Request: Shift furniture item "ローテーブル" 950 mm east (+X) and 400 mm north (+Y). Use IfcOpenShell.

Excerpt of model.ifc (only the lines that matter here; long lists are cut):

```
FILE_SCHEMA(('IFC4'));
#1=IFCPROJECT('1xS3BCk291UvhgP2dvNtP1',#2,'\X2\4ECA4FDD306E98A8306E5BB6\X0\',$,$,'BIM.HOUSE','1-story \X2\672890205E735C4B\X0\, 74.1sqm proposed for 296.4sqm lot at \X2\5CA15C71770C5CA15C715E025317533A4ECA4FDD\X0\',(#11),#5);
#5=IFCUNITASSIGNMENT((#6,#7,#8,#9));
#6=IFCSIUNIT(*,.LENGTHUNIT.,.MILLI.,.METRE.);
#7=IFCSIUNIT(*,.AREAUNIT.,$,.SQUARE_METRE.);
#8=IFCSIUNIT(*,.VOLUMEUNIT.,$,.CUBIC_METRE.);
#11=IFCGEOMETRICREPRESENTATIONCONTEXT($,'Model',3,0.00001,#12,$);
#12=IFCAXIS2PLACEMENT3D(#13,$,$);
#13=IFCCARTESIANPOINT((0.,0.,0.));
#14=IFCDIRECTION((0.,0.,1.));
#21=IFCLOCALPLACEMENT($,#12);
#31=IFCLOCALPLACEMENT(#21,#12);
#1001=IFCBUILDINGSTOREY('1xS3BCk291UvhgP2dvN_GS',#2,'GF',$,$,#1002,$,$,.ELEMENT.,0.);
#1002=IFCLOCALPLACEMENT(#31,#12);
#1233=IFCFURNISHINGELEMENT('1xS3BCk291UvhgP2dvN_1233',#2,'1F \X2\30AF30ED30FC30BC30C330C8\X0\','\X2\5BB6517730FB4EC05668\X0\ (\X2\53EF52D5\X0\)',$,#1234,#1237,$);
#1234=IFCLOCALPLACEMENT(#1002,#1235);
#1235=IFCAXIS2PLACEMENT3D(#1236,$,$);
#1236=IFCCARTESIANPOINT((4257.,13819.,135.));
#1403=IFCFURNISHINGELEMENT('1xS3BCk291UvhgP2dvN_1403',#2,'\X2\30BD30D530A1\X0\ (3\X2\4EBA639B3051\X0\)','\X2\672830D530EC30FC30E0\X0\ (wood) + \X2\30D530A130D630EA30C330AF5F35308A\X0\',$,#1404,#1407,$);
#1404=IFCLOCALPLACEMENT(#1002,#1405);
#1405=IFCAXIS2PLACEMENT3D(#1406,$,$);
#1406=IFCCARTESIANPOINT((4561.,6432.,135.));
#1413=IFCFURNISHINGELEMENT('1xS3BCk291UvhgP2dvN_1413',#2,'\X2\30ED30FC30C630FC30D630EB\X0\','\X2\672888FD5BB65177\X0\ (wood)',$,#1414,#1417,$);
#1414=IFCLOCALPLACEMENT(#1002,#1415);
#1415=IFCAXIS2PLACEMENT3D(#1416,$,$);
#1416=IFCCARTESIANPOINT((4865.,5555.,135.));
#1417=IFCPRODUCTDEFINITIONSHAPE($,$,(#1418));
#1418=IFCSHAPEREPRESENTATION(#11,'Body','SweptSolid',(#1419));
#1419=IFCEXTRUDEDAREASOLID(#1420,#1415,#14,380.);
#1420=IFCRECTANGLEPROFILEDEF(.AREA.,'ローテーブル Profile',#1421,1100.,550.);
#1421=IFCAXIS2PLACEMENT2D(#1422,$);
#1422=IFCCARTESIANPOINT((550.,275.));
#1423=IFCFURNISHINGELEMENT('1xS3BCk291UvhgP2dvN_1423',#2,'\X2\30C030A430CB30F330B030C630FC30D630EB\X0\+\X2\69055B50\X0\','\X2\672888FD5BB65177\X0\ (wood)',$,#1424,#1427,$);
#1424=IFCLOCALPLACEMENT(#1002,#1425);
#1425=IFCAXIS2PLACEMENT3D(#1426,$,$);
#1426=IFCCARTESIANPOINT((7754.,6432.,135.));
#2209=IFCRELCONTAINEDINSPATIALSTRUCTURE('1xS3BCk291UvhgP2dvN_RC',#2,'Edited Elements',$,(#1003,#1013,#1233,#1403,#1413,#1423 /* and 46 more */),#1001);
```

```python
import ifcopenshell
import ifcopenshell.api.geometry
import ifcopenshell.util.placement

model = ifcopenshell.open("model.ifc")

item = model.by_id(1413)
matrix = ifcopenshell.util.placement.get_local_placement(item.ObjectPlacement)
matrix[0, 3] += 950.0
matrix[1, 3] += 400.0
ifcopenshell.api.geometry.edit_object_placement(model, product=item, matrix=matrix, is_si=False)

print(ifcopenshell.util.placement.get_local_placement(item.ObjectPlacement).round(3) + 0.0)

model.write("model_v2.ifc")
```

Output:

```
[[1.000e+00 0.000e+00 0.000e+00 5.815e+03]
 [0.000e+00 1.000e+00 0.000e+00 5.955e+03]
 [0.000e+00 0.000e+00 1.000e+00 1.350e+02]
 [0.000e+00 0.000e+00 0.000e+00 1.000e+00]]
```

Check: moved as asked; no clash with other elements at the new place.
